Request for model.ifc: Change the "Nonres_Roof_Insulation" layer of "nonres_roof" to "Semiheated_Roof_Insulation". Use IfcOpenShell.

First a look at what the model holds.

```python
import ifcopenshell
import ifcopenshell.util.element

model = ifcopenshell.open("model.ifc")
print(model.schema)
for layer_set in model.by_type("IfcMaterialLayerSet"):
    if layer_set.LayerSetName == "nonres_roof":
        for layer in layer_set.MaterialLayers:
            print(layer.id(), layer.Material and layer.Material.Name, layer.LayerThickness, sep=" | ")
        print(len(ifcopenshell.util.element.get_elements_by_material(model, layer_set)), "elements and types use it")
print(sorted(m.Name for m in model.by_type("IfcMaterial") if m.Name)[:60])
```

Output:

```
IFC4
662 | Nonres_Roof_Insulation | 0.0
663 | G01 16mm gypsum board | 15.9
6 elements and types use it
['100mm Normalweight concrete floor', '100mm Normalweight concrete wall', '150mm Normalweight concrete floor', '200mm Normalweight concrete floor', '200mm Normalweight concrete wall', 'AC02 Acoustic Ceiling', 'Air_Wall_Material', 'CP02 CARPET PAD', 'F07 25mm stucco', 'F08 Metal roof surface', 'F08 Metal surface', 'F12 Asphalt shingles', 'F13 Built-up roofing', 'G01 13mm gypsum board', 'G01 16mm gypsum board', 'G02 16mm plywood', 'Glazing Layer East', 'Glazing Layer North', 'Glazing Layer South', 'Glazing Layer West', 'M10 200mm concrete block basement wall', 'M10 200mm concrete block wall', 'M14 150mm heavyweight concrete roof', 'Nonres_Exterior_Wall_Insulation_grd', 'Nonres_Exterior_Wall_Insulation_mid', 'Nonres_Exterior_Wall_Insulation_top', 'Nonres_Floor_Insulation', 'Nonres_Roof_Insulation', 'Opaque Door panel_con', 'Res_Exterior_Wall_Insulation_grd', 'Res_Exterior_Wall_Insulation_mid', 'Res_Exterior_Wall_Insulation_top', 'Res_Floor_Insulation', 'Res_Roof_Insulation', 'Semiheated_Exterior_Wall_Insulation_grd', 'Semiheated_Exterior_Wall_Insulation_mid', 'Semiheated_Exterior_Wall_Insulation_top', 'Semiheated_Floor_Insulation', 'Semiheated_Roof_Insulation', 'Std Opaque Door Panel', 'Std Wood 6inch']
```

```python
import ifcopenshell
import ifcopenshell.api.material

model = ifcopenshell.open("model.ifc")

layer_set = next(s for s in model.by_type("IfcMaterialLayerSet") if s.LayerSetName == "nonres_roof")
layer = next(l for l in layer_set.MaterialLayers if l.Material and l.Material.Name == "Nonres_Roof_Insulation")
material = next(m for m in model.by_type("IfcMaterial") if m.Name == "Semiheated_Roof_Insulation")

# Point this one layer at the other material; renaming the old one would change it everywhere.
ifcopenshell.api.material.edit_layer(model, layer=layer, attributes={}, material=material)

print([l.Material.Name if l.Material else None for l in layer_set.MaterialLayers])

model.write("model_edited.ifc")
```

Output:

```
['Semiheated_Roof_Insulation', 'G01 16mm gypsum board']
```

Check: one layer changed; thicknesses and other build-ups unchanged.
